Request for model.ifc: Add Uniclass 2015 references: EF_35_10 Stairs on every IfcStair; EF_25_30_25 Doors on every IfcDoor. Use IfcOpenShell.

First a look at what the model holds.

```python
import ifcopenshell

model = ifcopenshell.open("model.ifc")
print(model.schema)
print("classifications:", [c.Name for c in model.by_type("IfcClassification")])
for ifc_class in ("IfcDoor", "IfcRoof", "IfcStair", "IfcWall", "IfcWindow"):
    print(ifc_class, len(model.by_type(ifc_class)))
```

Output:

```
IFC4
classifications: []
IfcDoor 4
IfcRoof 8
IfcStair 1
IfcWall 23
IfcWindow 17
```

```python
import ifcopenshell
import ifcopenshell.api.classification

model = ifcopenshell.open("model.ifc")

system = ifcopenshell.api.classification.add_classification(model, classification="Uniclass 2015")

codes = {
    "IfcStair": ("EF_35_10", "Stairs"),
    "IfcDoor": ("EF_25_30_25", "Doors"),
}
for ifc_class, (code, name) in codes.items():
    products = model.by_type(ifc_class)
    ifcopenshell.api.classification.add_reference(
        model, products=products, classification=system, identification=code, name=name
    )
    print(code, len(products))

model.write("model_rev.ifc")
```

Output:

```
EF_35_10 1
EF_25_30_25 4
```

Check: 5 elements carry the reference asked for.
